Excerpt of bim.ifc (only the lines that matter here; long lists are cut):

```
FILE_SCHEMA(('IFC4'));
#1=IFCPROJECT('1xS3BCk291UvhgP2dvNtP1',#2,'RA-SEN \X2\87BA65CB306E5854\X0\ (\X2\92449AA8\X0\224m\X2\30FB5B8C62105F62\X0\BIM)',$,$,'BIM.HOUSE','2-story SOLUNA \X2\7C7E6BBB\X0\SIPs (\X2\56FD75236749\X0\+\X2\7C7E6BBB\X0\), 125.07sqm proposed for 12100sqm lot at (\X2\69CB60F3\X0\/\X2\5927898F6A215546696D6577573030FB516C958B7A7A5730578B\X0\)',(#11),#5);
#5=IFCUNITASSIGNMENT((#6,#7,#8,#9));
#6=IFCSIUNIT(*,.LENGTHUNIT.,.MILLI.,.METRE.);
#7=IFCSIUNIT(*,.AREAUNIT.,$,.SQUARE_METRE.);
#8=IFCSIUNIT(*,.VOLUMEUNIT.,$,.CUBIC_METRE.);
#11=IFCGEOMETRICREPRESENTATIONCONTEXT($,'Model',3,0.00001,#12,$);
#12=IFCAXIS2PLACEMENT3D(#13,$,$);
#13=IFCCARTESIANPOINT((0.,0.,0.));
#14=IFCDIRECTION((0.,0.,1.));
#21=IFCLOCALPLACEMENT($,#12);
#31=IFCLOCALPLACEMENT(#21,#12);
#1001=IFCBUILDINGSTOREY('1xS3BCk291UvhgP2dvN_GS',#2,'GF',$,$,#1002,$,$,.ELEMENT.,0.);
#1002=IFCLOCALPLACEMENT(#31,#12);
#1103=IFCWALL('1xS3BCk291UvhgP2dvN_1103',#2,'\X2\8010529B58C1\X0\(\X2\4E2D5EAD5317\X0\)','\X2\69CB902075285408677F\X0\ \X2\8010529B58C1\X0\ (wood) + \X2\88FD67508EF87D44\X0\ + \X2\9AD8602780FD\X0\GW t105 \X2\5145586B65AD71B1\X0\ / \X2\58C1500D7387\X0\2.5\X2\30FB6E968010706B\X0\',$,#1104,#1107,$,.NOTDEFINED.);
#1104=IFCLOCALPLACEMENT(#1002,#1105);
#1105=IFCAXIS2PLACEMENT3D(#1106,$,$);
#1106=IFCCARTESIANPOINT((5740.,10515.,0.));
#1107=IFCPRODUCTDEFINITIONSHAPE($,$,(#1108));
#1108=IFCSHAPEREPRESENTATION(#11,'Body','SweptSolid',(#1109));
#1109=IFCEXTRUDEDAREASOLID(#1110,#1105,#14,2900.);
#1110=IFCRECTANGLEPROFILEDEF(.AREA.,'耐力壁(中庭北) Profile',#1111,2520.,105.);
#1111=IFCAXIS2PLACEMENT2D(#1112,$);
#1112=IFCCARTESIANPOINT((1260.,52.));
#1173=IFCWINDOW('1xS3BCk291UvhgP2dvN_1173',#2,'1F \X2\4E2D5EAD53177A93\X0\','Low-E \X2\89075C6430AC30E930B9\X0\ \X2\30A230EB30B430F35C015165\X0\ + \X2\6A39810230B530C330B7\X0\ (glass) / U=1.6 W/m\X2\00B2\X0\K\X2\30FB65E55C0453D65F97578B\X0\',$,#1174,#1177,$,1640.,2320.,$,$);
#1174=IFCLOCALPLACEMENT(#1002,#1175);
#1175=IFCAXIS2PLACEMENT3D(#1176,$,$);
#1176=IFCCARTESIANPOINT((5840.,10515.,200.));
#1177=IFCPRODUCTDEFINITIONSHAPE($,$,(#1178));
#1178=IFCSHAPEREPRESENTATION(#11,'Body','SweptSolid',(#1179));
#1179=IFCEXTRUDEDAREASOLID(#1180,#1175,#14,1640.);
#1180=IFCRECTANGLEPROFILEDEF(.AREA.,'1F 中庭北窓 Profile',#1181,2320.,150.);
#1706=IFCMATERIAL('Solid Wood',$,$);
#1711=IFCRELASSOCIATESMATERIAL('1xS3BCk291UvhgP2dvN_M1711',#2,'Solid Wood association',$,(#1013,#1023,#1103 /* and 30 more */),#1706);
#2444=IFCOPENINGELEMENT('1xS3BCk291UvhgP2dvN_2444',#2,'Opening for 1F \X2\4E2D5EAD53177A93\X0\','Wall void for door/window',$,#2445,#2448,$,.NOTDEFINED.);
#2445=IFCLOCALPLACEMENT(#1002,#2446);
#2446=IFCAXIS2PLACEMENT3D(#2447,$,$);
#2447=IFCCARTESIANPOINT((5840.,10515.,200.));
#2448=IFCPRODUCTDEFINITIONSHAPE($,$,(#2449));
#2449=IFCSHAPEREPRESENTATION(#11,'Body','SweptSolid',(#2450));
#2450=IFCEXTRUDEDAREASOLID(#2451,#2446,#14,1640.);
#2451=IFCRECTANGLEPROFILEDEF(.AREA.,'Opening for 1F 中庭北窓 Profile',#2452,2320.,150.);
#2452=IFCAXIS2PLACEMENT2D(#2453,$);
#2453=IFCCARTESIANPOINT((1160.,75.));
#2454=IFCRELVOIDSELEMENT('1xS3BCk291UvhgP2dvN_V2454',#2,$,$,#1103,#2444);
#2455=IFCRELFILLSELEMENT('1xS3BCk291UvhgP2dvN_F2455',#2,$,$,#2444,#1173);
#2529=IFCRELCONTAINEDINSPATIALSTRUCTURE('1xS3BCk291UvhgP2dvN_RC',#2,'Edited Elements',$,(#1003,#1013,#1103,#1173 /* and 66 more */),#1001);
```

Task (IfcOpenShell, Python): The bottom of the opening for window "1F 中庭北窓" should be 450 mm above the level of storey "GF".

```python
import numpy as np
import ifcopenshell
import ifcopenshell.api.geometry
import ifcopenshell.geom
import ifcopenshell.util.element
import ifcopenshell.util.placement
import ifcopenshell.util.shape
import ifcopenshell.util.unit

model = ifcopenshell.open("bim.ifc")
unit_scale = ifcopenshell.util.unit.calculate_unit_scale(model)

window = model.by_guid("1xS3BCk291UvhgP2dvN_1173")
opening = window.FillsVoids[0].RelatingOpeningElement
storey = ifcopenshell.util.element.get_container(window, ifc_class="IfcBuildingStorey")
level = ifcopenshell.util.placement.get_local_placement(storey.ObjectPlacement)[2, 3]

# The opening's origin need not be at the sill, so measure its lowest point.
shape = ifcopenshell.geom.create_shape(ifcopenshell.geom.settings(), opening)
bottom = ifcopenshell.util.shape.get_shape_bottom_elevation(shape, shape.geometry) / unit_scale
dz = level + 0.45 / unit_scale - bottom

shift = np.array([0.0, 0.0, dz])
# The window is not placed relative to its opening, so move both.
for product in (opening, window):
    matrix = ifcopenshell.util.placement.get_local_placement(product.ObjectPlacement)
    matrix[:3, 3] += shift
    ifcopenshell.api.geometry.edit_object_placement(model, product=product, matrix=matrix, is_si=False)

print(f"moved by {dz * unit_scale:+.3f} m")

model.write("bim-out.ifc")
```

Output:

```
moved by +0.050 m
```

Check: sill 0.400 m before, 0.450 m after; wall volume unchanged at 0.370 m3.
